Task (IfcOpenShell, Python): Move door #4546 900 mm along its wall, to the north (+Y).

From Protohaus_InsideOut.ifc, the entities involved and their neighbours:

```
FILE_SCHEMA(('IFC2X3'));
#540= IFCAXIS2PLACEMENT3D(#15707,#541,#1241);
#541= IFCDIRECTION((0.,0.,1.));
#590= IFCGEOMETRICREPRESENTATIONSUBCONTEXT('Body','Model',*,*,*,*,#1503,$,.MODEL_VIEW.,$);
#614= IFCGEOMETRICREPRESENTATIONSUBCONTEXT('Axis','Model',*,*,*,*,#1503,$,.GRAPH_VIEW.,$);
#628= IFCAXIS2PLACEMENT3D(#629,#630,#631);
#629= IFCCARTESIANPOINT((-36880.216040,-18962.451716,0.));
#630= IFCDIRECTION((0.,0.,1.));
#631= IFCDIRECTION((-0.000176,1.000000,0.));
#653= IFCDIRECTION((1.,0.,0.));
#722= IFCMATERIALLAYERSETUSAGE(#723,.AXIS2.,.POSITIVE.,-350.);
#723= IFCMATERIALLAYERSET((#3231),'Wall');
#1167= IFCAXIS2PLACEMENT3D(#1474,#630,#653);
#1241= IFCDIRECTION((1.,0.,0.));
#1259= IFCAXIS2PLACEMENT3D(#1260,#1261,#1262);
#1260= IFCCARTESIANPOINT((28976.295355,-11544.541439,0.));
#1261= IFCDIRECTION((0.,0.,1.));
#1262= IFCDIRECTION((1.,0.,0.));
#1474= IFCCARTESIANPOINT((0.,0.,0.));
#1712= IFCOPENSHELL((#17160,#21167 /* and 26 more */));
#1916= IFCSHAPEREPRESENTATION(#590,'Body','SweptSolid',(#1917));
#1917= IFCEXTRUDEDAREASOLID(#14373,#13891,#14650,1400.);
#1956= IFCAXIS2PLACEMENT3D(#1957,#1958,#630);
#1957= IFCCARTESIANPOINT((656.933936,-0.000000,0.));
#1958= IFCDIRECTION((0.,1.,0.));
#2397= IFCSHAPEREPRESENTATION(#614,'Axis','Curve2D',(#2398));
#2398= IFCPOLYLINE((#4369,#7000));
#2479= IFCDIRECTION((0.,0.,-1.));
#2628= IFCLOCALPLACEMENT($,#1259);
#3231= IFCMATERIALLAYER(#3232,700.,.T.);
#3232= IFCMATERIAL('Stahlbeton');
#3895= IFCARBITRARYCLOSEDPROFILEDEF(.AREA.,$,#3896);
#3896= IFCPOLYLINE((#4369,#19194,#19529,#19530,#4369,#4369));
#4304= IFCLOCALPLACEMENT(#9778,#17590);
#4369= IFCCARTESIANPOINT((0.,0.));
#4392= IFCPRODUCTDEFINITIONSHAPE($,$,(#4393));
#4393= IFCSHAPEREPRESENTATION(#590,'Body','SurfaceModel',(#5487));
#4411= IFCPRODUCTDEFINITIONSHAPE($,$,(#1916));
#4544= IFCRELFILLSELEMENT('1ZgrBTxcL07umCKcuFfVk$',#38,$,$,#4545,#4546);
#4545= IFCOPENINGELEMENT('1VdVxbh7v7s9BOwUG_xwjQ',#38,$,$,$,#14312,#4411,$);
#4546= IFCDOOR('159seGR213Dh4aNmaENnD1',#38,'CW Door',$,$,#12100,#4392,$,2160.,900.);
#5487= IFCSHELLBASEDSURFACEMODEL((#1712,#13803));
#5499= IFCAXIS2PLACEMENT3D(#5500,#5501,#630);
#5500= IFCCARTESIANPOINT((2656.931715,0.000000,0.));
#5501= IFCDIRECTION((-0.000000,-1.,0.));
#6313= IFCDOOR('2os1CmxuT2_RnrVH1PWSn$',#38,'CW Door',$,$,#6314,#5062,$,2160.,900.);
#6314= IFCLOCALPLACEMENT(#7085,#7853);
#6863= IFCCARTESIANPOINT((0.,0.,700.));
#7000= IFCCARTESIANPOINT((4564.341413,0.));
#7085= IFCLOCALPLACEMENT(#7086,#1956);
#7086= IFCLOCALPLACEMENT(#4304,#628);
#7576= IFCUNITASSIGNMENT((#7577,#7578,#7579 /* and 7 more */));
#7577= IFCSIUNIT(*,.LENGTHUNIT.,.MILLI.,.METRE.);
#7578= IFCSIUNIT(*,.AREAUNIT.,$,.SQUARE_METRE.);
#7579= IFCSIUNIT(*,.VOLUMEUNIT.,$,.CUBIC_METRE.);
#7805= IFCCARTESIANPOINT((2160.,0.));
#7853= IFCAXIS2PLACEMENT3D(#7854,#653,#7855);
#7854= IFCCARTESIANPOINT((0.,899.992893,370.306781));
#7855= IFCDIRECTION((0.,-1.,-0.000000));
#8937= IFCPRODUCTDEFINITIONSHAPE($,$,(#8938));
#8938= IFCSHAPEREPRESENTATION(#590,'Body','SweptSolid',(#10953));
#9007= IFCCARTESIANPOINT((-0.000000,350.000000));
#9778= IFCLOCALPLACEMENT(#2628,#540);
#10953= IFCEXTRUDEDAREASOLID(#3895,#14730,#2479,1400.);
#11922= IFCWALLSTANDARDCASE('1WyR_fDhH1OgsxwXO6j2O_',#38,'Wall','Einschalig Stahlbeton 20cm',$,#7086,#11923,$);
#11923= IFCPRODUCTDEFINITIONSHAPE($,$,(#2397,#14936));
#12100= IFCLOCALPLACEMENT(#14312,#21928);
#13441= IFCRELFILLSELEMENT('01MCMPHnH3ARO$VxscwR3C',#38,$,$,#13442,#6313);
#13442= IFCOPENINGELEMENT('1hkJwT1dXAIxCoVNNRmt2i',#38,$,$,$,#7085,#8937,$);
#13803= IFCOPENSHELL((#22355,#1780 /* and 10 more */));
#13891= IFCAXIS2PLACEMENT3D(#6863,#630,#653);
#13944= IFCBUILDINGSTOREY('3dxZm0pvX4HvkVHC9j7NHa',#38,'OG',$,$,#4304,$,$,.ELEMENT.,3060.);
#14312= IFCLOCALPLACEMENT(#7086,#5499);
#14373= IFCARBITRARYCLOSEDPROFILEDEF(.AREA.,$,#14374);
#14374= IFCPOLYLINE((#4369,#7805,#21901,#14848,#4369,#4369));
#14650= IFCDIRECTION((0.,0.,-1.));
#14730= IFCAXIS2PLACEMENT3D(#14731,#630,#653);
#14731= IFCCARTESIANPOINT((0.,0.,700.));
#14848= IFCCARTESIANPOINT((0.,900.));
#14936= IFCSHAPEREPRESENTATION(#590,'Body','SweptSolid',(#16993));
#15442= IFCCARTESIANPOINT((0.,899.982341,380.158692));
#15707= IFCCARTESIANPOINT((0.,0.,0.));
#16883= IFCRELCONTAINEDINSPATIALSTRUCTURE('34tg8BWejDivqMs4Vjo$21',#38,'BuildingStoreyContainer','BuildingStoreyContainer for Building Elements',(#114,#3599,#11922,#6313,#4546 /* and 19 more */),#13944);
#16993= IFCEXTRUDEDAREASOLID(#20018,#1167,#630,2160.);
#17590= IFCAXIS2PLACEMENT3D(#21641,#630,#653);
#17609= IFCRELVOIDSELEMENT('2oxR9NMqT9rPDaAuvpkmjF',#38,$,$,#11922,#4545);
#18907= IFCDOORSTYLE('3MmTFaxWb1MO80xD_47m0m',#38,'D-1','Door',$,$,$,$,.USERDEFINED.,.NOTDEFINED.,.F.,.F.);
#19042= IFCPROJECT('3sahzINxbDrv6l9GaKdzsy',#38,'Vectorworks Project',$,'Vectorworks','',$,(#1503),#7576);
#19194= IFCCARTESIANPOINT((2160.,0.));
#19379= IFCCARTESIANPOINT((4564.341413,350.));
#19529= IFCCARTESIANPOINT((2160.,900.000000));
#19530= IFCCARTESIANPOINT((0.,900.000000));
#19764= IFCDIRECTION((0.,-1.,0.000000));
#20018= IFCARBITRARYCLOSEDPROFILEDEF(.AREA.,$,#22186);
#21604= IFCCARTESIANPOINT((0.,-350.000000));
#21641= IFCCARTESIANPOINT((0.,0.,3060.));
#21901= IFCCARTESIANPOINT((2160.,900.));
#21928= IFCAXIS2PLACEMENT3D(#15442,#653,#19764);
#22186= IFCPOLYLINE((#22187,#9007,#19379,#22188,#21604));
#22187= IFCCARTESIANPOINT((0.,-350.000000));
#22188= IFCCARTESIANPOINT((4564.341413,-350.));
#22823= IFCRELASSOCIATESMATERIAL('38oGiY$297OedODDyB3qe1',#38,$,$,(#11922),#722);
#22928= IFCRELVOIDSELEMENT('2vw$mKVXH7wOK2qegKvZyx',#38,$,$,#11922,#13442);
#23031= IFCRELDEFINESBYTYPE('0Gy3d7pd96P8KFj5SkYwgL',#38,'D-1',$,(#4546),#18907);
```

```python
import ifcopenshell
import ifcopenshell.api.geometry
import ifcopenshell.util.placement

model = ifcopenshell.open("Protohaus_InsideOut.ifc")

door = model.by_id(4546)
opening = door.FillsVoids[0].RelatingOpeningElement
wall = opening.VoidsElements[0].RelatingBuildingElement

wall_matrix = ifcopenshell.util.placement.get_local_placement(wall.ObjectPlacement)
shift = wall_matrix[:3, 0] * 900.0
before = ifcopenshell.util.placement.get_local_placement(door.ObjectPlacement)[:3, 3].copy()

# The door is placed relative to its opening, so it follows when the opening moves.
matrix = ifcopenshell.util.placement.get_local_placement(opening.ObjectPlacement)
matrix[:3, 3] += shift
ifcopenshell.api.geometry.edit_object_placement(
    model, product=opening, matrix=matrix, is_si=False, should_transform_children=True
)

after = ifcopenshell.util.placement.get_local_placement(door.ObjectPlacement)[:3, 3]
print("door moved by", (after - before).round(3) + 0.0)

model.write("Protohaus_InsideOut_v2.ifc")
```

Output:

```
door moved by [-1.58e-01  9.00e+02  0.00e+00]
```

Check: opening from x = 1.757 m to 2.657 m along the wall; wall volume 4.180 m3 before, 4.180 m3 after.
